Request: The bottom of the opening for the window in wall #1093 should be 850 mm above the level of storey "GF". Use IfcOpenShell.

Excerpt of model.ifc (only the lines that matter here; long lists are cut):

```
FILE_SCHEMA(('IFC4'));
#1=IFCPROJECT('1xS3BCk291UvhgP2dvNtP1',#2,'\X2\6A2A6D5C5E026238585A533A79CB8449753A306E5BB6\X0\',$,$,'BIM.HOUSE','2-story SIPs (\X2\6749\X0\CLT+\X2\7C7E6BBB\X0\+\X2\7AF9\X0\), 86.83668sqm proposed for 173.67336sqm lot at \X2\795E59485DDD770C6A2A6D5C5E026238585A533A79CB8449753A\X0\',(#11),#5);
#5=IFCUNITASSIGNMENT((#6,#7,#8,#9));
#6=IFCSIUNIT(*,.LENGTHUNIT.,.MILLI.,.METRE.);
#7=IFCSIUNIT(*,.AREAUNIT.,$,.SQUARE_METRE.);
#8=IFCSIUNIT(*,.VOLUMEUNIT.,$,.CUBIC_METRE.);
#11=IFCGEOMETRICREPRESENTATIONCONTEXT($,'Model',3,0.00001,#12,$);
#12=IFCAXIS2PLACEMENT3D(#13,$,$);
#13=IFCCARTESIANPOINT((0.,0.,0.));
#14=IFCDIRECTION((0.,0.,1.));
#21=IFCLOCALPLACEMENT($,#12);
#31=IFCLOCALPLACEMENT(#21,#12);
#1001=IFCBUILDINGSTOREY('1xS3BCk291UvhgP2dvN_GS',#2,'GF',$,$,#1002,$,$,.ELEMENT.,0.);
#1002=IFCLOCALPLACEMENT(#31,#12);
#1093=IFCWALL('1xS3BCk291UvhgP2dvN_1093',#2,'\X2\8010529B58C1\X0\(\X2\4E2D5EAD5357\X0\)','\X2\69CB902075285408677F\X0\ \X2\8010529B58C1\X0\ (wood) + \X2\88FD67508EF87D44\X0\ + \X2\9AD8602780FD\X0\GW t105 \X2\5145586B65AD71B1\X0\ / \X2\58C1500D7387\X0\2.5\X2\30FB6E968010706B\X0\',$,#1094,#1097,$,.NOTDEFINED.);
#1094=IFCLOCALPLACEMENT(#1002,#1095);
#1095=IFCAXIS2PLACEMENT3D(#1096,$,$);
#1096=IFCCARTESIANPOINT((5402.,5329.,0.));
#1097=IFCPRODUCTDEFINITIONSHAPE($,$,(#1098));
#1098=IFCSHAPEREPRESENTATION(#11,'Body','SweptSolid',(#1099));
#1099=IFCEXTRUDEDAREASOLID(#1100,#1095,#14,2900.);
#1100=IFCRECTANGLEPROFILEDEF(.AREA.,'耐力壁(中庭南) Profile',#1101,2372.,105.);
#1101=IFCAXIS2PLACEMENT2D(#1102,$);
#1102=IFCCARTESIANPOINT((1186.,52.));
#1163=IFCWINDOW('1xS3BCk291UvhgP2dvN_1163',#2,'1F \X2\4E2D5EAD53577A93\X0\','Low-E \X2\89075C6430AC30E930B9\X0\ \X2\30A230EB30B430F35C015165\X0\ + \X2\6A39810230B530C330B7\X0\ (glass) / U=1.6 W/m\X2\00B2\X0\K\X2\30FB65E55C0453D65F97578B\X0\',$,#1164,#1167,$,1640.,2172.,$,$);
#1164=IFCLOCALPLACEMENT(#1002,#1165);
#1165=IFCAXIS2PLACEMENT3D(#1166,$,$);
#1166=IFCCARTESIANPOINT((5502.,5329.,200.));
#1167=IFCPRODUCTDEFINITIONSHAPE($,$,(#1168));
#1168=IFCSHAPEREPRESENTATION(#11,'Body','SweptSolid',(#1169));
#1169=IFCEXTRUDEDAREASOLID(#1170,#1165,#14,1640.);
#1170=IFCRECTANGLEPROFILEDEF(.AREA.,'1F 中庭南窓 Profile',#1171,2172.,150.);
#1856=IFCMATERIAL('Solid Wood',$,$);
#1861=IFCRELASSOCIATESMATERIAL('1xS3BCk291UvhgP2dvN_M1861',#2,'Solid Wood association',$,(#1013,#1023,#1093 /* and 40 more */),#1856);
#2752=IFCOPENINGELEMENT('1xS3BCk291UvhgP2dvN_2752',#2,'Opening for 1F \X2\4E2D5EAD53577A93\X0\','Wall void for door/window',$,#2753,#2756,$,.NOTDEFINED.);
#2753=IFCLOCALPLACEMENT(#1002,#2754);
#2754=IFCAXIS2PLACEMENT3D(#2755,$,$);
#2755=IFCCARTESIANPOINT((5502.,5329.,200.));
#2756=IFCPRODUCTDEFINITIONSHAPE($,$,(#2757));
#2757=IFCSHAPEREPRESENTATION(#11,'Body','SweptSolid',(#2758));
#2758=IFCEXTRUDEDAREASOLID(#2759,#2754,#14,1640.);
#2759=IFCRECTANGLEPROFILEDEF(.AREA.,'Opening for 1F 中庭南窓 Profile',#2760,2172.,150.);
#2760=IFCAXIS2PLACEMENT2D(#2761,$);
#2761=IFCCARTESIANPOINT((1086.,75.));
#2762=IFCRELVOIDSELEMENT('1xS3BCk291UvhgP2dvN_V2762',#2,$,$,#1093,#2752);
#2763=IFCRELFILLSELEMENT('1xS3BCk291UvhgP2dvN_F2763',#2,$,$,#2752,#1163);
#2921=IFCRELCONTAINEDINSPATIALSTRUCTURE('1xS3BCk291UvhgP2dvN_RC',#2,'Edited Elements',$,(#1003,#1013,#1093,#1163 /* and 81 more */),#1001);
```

```python
import numpy as np
import ifcopenshell
import ifcopenshell.api.geometry
import ifcopenshell.geom
import ifcopenshell.util.element
import ifcopenshell.util.placement
import ifcopenshell.util.shape
import ifcopenshell.util.unit

model = ifcopenshell.open("model.ifc")
unit_scale = ifcopenshell.util.unit.calculate_unit_scale(model)

window = model.by_guid("1xS3BCk291UvhgP2dvN_1163")
opening = window.FillsVoids[0].RelatingOpeningElement
storey = ifcopenshell.util.element.get_container(window, ifc_class="IfcBuildingStorey")
level = ifcopenshell.util.placement.get_local_placement(storey.ObjectPlacement)[2, 3]

# The opening's origin need not be at the sill, so measure its lowest point.
shape = ifcopenshell.geom.create_shape(ifcopenshell.geom.settings(), opening)
bottom = ifcopenshell.util.shape.get_shape_bottom_elevation(shape, shape.geometry) / unit_scale
dz = level + 0.85 / unit_scale - bottom

shift = np.array([0.0, 0.0, dz])
# The window is not placed relative to its opening, so move both.
for product in (opening, window):
    matrix = ifcopenshell.util.placement.get_local_placement(product.ObjectPlacement)
    matrix[:3, 3] += shift
    ifcopenshell.api.geometry.edit_object_placement(model, product=product, matrix=matrix, is_si=False)

print(f"moved by {dz * unit_scale:+.3f} m")

model.write("model_updated.ifc")
```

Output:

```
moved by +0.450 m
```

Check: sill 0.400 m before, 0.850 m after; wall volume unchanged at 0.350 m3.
